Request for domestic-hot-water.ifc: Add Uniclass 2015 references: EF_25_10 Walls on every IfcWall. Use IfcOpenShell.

First a look at what the model holds.

```python
import ifcopenshell

model = ifcopenshell.open("domestic-hot-water.ifc")
print(model.schema)
print("classifications:", [c.Name for c in model.by_type("IfcClassification")])
for ifc_class in ("IfcDoor", "IfcRoof", "IfcStair", "IfcWall", "IfcWindow"):
    print(ifc_class, len(model.by_type(ifc_class)))
```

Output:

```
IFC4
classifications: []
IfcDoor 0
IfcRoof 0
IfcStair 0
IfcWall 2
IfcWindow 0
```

```python
import ifcopenshell
import ifcopenshell.api.classification

model = ifcopenshell.open("domestic-hot-water.ifc")

system = ifcopenshell.api.classification.add_classification(model, classification="Uniclass 2015")

codes = {
    "IfcWall": ("EF_25_10", "Walls"),
}
for ifc_class, (code, name) in codes.items():
    products = model.by_type(ifc_class)
    ifcopenshell.api.classification.add_reference(
        model, products=products, classification=system, identification=code, name=name
    )
    print(code, len(products))

model.write("domestic-hot-water_rev.ifc")
```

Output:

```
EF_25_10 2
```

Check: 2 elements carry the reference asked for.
